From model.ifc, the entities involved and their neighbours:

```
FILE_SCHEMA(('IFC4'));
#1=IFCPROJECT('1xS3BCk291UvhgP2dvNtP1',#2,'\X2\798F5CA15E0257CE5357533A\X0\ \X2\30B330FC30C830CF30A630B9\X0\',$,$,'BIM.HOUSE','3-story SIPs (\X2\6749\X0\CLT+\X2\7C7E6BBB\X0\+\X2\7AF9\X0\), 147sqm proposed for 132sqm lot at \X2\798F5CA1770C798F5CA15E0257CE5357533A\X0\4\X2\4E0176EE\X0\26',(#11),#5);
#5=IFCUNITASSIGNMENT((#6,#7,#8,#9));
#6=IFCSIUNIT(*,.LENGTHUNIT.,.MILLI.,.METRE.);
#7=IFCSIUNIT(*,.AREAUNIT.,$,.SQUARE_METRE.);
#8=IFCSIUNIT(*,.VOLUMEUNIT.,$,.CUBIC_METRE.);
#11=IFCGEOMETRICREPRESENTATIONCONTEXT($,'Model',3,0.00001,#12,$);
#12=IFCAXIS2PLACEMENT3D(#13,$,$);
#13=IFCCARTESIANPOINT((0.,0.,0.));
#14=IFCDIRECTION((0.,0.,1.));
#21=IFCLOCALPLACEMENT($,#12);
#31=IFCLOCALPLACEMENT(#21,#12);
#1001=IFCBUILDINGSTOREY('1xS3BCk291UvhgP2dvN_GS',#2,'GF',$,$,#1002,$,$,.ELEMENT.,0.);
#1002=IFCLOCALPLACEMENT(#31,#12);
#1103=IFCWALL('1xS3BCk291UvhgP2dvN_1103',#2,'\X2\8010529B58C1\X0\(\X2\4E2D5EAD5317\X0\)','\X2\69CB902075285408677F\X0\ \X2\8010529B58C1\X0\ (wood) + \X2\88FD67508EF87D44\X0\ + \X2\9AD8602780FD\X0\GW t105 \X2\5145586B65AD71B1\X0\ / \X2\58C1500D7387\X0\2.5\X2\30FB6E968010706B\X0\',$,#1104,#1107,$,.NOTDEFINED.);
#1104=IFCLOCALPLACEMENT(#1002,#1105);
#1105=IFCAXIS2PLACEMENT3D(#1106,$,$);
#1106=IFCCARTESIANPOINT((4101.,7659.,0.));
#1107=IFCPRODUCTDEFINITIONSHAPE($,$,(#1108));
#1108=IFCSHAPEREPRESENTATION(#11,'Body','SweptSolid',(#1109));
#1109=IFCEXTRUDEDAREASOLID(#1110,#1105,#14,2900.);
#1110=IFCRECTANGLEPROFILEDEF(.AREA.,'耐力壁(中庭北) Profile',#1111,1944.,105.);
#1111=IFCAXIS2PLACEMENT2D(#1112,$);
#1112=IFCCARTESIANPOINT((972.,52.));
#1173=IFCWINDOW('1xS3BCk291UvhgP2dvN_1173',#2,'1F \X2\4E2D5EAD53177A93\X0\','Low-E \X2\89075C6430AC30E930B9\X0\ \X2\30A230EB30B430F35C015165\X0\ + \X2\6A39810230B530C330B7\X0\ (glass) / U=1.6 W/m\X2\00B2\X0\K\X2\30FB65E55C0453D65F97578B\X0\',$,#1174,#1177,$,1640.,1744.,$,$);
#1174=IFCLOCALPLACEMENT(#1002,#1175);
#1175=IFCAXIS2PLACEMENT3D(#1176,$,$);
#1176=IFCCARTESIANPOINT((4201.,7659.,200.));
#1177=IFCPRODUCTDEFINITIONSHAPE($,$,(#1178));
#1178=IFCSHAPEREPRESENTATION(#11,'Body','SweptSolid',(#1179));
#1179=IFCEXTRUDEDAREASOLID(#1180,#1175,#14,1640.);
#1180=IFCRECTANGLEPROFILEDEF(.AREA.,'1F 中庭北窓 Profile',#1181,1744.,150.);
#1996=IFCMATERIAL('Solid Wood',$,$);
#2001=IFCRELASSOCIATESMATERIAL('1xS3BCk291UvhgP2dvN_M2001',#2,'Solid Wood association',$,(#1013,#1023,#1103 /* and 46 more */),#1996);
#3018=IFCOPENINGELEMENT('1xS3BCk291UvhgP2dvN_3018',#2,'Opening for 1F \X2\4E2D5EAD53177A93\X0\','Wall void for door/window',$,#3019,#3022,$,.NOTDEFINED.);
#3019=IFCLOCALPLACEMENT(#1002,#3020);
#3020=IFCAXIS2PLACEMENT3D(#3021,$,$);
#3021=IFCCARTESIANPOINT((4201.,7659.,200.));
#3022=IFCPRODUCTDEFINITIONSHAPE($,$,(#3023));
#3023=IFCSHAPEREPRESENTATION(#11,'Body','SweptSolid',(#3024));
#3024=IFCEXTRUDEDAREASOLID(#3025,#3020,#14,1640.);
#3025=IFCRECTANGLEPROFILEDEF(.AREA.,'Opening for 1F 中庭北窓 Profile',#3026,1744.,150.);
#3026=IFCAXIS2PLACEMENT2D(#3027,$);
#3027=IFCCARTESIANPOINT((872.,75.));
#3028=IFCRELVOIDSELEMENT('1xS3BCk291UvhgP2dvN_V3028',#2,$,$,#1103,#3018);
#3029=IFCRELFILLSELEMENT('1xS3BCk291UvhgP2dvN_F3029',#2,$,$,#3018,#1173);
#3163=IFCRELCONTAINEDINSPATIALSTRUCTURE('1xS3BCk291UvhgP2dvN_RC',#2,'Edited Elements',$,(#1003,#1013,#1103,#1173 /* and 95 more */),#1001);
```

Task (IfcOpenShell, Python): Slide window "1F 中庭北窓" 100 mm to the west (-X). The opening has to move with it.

```python
import ifcopenshell
import ifcopenshell.api.geometry
import ifcopenshell.util.placement

model = ifcopenshell.open("model.ifc")

window = model.by_guid("1xS3BCk291UvhgP2dvN_1173")
opening = window.FillsVoids[0].RelatingOpeningElement
wall = opening.VoidsElements[0].RelatingBuildingElement

wall_matrix = ifcopenshell.util.placement.get_local_placement(wall.ObjectPlacement)
shift = wall_matrix[:3, 0] * -100.0
before = ifcopenshell.util.placement.get_local_placement(window.ObjectPlacement)[:3, 3].copy()

# The window is not placed relative to its opening, so move both.
for product in (opening, window):
    matrix = ifcopenshell.util.placement.get_local_placement(product.ObjectPlacement)
    matrix[:3, 3] += shift
    ifcopenshell.api.geometry.edit_object_placement(model, product=product, matrix=matrix, is_si=False)

after = ifcopenshell.util.placement.get_local_placement(window.ObjectPlacement)[:3, 3]
print("window moved by", (after - before).round(3) + 0.0)

model.write("model-out.ifc")
```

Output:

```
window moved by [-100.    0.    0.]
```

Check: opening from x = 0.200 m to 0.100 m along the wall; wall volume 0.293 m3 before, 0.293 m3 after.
